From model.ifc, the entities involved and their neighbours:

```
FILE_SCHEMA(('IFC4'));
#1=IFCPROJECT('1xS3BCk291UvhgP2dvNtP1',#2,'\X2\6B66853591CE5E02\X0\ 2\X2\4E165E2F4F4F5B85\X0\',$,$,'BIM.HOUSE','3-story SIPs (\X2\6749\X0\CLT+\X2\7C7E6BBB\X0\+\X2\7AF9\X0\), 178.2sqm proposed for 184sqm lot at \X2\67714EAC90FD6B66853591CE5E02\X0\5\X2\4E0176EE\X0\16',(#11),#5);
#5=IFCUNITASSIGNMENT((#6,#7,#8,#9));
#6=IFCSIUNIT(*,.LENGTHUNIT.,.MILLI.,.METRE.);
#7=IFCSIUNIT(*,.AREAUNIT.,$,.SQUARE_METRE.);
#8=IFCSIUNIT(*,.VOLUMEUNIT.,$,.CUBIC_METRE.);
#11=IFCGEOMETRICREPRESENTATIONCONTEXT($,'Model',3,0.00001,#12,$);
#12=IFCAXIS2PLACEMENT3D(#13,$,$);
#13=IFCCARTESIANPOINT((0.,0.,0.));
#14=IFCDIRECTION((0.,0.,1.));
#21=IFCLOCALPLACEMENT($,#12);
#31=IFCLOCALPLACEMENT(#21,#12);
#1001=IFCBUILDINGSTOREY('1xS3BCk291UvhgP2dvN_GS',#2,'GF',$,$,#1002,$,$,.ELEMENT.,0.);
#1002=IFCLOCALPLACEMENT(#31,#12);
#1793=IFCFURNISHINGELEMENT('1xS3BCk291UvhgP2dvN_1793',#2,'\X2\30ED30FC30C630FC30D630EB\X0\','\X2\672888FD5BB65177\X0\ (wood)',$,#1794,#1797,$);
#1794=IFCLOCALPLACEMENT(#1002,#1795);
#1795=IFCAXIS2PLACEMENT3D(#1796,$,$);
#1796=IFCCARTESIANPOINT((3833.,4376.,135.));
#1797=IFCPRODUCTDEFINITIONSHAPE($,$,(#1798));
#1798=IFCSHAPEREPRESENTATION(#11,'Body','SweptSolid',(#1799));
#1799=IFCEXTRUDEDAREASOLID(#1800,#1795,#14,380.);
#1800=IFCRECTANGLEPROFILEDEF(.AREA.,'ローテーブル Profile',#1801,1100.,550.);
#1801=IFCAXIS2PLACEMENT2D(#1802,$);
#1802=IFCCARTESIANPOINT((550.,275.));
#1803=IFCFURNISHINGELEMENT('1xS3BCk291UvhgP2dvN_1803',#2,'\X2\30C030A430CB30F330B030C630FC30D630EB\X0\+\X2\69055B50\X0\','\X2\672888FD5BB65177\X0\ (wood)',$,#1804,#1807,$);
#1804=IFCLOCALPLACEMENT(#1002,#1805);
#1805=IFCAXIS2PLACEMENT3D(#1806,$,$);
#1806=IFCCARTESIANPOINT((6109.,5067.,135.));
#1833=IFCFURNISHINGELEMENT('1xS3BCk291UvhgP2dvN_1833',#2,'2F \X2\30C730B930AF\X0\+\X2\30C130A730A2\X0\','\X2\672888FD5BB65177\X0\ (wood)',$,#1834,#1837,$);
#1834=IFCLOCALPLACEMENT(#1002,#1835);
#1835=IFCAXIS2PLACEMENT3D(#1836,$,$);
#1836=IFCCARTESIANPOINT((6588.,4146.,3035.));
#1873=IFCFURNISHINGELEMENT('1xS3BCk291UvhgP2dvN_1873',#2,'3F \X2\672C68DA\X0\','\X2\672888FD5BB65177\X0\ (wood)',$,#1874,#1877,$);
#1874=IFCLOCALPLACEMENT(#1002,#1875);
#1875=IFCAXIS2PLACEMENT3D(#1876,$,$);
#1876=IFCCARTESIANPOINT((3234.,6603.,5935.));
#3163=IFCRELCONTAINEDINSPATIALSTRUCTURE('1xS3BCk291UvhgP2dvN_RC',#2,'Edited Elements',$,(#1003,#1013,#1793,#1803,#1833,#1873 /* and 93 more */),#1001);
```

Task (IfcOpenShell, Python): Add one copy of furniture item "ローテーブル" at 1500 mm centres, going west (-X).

```python
import numpy as np
import ifcopenshell
import ifcopenshell.api.geometry
import ifcopenshell.api.root
import ifcopenshell.util.element
import ifcopenshell.util.placement
import ifcopenshell.util.unit

model = ifcopenshell.open("model.ifc")
unit_scale = ifcopenshell.util.unit.calculate_unit_scale(model)


def reuse_history(source, copy):
    """copy_class also copies each property set's owner history, people and application; keep the originals."""
    for rel in copy.IsDefinedBy:
        if rel.is_a("IfcRelDefinesByProperties") and (history := rel.RelatingPropertyDefinition.OwnerHistory):
            rel.RelatingPropertyDefinition.OwnerHistory = source.OwnerHistory
            ifcopenshell.util.element.remove_deep2(model, history)


source = model.by_id(1793)
base = ifcopenshell.util.placement.get_local_placement(source.ObjectPlacement)
step = np.array([-1.0, 0.0, 0.0]) * 1.5 / unit_scale

for i in range(1, 2):
    copy = ifcopenshell.api.root.copy_class(model, product=source)
    copy.Representation = ifcopenshell.util.element.copy_deep(
        model, source.Representation, exclude=["IfcGeometricRepresentationContext", "IfcRepresentationMap"]
    )
    reuse_history(source, copy)
    matrix = base.copy()
    matrix[:3, 3] += i * step
    print("added at", matrix[:3, 3].round(3) + 0.0)
    ifcopenshell.api.geometry.edit_object_placement(model, product=copy, matrix=matrix, is_si=False)

model.write("model_v2.ifc")
```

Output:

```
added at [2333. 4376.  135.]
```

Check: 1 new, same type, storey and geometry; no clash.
